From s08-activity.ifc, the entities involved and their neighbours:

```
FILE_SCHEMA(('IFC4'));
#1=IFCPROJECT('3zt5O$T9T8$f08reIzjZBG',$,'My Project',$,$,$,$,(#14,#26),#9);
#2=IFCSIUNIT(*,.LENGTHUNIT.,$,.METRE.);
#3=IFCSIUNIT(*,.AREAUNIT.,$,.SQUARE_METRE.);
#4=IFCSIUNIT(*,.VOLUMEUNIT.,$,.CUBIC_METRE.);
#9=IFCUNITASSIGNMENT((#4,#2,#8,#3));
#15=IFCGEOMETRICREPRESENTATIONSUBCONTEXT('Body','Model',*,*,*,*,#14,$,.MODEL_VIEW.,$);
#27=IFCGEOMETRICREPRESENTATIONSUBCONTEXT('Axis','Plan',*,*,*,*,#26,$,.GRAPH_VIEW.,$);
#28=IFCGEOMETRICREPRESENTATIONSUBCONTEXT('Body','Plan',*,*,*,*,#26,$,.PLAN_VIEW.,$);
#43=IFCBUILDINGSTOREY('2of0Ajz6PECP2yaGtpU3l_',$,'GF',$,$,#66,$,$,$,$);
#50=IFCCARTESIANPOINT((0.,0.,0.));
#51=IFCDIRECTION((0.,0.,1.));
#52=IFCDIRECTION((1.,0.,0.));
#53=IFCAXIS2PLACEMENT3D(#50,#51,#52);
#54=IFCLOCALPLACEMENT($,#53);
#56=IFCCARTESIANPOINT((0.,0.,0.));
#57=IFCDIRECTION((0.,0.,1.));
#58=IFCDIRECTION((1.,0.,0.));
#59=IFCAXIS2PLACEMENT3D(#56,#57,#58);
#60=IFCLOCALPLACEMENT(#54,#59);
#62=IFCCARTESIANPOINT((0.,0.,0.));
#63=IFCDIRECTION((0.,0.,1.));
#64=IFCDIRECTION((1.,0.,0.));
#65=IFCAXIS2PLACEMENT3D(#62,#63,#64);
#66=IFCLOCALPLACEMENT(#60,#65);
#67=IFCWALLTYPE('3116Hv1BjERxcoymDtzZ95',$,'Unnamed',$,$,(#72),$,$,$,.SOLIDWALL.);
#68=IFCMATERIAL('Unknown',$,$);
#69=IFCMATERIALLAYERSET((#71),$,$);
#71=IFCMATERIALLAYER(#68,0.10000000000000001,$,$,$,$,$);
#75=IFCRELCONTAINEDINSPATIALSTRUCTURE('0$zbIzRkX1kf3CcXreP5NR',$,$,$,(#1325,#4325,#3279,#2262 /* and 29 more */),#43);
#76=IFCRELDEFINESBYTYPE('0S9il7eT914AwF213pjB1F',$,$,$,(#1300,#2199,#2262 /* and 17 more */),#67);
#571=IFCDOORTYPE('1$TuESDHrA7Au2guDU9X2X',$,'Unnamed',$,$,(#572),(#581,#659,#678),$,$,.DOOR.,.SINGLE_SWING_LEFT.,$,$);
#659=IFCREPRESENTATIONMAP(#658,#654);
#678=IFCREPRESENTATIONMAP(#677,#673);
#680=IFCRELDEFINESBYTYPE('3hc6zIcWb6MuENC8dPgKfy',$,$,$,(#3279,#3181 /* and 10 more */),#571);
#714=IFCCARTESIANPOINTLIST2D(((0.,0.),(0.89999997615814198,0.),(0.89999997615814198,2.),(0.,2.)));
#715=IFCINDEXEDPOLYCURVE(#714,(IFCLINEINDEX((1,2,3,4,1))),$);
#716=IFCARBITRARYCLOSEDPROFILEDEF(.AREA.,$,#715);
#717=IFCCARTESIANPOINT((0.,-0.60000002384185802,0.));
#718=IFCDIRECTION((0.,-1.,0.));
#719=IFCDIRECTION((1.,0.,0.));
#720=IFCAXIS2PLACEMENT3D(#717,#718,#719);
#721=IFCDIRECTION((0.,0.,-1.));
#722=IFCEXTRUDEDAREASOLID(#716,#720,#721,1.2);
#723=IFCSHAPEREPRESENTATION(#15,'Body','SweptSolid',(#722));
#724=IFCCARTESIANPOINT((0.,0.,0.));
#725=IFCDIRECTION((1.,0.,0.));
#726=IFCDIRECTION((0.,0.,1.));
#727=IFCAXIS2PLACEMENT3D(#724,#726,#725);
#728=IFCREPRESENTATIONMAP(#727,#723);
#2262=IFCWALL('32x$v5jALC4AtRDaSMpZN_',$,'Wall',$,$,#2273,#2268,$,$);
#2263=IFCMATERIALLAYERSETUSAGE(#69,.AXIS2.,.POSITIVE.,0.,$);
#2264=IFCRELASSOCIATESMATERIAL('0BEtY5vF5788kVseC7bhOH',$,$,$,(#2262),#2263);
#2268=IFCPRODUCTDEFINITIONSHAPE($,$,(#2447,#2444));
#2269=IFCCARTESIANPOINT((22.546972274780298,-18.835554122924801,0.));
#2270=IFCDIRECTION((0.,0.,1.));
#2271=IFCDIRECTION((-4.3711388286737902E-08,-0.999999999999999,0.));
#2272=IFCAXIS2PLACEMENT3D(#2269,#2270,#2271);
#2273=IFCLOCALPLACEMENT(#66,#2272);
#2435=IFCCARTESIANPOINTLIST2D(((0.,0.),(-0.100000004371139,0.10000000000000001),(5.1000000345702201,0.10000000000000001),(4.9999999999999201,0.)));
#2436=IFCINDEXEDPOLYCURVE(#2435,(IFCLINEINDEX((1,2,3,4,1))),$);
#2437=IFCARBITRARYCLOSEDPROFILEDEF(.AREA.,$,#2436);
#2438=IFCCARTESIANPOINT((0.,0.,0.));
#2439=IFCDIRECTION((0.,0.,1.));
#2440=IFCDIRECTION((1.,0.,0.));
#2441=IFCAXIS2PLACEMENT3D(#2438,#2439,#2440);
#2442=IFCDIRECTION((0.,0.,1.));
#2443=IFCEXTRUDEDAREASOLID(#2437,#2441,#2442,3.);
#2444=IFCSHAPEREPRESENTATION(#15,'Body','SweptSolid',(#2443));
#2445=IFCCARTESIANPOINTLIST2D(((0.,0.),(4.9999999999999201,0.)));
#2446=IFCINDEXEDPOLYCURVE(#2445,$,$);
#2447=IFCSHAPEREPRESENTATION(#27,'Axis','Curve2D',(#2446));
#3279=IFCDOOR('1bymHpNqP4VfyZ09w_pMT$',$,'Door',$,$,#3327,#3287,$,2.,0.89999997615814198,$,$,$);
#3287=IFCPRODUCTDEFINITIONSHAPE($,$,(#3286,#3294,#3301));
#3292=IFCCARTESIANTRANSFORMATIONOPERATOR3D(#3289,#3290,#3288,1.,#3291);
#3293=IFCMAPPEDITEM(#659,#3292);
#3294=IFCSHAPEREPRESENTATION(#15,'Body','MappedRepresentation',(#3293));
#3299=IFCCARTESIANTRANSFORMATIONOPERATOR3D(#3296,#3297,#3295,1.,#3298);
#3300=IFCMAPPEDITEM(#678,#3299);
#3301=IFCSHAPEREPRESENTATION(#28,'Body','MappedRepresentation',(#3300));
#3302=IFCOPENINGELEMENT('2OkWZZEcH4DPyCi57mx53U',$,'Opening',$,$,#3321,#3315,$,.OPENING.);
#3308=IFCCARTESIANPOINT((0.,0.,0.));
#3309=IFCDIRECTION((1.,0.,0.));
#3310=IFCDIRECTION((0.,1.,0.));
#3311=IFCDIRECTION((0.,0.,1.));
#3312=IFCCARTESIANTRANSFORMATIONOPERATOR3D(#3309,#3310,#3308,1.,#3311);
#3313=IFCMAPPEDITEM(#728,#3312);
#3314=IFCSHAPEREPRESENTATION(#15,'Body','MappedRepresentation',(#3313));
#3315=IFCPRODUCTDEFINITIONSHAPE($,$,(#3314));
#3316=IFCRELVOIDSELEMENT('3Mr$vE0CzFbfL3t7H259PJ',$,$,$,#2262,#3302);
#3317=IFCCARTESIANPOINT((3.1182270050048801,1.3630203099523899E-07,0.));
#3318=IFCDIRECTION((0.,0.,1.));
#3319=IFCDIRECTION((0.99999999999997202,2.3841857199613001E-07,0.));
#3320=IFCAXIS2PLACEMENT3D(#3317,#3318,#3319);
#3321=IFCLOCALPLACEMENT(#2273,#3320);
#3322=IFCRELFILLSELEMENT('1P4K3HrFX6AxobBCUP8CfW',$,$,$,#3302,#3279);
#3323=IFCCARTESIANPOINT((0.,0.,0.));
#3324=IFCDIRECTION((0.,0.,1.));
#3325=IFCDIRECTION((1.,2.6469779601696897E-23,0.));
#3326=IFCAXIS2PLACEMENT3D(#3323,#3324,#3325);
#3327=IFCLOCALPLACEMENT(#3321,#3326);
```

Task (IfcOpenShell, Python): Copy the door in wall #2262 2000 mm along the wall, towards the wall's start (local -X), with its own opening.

```python
import ifcopenshell
import ifcopenshell.api.feature
import ifcopenshell.api.geometry
import ifcopenshell.api.root
import ifcopenshell.geom
import ifcopenshell.util.element
import ifcopenshell.util.placement
import ifcopenshell.util.shape

model = ifcopenshell.open("s08-activity.ifc")
settings = ifcopenshell.geom.settings()


def volume(element):
    """Net volume in cubic metres, openings subtracted."""
    shape = ifcopenshell.geom.create_shape(settings, element)
    return ifcopenshell.util.shape.get_volume(shape.geometry)


door = model.by_guid("1bymHpNqP4VfyZ09w_pMT$")
opening = door.FillsVoids[0].RelatingOpeningElement
wall = opening.VoidsElements[0].RelatingBuildingElement
before = volume(wall)
shift = ifcopenshell.util.placement.get_local_placement(wall.ObjectPlacement)[:3, 0] * -2.0

# copy_class copies the void relationship, type, container and properties, but no geometry.
new_opening = ifcopenshell.api.root.copy_class(model, product=opening)
new_opening.Representation = ifcopenshell.util.element.copy_deep(
    model, opening.Representation, exclude=["IfcGeometricRepresentationContext", "IfcRepresentationMap"]
)
new_door = ifcopenshell.api.root.copy_class(model, product=door)
new_door.Representation = ifcopenshell.util.element.copy_deep(
    model, door.Representation, exclude=["IfcGeometricRepresentationContext", "IfcRepresentationMap"]
)
ifcopenshell.api.feature.add_filling(model, opening=new_opening, element=new_door)

for old, new in ((opening, new_opening), (door, new_door)):
    matrix = ifcopenshell.util.placement.get_local_placement(old.ObjectPlacement)
    matrix[:3, 3] += shift
    ifcopenshell.api.geometry.edit_object_placement(model, product=new, matrix=matrix, is_si=False)

after = volume(wall)

print(f"wall volume {before:.3f} -> {after:.3f} m3")

model.write("s08-activity_v2.ifc")
```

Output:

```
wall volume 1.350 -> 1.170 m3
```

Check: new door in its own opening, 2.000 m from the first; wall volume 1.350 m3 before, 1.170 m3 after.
